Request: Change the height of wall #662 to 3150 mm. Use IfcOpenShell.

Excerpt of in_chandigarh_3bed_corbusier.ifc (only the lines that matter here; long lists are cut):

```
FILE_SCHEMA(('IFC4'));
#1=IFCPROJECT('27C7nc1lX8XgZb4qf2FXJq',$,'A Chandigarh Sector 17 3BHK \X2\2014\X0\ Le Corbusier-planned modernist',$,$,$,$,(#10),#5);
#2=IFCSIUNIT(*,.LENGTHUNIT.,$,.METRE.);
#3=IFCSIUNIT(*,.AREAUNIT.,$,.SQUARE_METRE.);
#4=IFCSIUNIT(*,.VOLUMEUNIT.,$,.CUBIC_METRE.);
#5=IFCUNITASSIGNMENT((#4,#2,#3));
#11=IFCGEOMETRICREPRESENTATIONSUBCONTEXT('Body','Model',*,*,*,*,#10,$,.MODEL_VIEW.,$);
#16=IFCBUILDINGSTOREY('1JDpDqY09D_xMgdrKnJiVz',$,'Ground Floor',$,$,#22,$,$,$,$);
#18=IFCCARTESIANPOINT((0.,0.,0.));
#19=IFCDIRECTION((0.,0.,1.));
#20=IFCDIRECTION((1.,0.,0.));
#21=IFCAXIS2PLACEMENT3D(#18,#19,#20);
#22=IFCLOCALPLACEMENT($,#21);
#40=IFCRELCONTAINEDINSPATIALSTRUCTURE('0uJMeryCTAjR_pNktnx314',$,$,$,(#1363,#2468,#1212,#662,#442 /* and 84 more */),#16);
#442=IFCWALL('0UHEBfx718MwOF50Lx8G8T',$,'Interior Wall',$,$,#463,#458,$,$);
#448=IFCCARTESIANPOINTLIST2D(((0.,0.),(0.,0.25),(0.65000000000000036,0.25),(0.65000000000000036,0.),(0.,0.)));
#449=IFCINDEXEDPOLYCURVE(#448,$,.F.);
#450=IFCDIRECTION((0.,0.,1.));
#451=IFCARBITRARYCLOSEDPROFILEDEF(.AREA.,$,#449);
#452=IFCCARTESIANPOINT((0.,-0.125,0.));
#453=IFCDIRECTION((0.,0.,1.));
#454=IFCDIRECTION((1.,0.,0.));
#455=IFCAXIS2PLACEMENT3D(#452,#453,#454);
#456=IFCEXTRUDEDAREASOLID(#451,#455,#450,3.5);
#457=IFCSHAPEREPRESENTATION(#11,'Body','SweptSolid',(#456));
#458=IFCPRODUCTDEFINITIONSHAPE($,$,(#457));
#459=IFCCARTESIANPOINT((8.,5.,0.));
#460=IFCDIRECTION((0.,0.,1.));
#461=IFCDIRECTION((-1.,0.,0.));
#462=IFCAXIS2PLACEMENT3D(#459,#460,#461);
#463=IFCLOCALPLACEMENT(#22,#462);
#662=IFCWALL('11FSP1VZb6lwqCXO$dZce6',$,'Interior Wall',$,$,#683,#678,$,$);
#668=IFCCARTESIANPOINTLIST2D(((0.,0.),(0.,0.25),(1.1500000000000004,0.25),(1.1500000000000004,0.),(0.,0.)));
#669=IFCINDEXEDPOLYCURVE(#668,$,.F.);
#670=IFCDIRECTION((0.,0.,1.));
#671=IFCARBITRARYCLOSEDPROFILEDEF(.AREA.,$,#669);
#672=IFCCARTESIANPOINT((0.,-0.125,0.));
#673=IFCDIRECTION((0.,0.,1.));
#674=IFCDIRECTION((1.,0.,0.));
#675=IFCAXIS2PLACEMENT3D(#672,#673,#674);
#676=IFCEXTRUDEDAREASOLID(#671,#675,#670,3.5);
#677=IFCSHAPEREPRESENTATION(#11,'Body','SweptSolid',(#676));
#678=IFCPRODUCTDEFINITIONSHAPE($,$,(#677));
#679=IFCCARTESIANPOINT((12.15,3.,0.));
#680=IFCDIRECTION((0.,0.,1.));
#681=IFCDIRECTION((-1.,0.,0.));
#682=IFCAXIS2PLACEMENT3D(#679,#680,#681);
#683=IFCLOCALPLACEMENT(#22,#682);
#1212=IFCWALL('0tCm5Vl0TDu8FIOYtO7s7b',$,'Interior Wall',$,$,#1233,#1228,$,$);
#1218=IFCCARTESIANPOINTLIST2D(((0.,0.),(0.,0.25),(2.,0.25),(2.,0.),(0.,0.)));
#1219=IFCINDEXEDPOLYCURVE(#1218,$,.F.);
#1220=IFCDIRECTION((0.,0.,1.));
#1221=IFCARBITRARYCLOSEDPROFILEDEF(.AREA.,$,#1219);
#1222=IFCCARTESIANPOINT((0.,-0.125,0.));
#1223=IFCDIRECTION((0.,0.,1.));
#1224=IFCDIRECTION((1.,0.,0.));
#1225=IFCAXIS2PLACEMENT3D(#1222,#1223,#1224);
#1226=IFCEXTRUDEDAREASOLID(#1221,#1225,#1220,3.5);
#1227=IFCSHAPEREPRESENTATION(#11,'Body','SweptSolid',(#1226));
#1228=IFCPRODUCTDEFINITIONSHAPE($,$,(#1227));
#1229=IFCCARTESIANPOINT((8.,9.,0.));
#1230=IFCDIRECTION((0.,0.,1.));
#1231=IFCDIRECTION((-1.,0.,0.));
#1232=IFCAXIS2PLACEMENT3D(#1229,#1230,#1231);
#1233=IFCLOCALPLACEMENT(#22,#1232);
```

```python
import ifcopenshell
import ifcopenshell.geom
import ifcopenshell.util.representation
import ifcopenshell.util.shape

model = ifcopenshell.open("in_chandigarh_3bed_corbusier.ifc")
settings = ifcopenshell.geom.settings()


def volume(element):
    """Net volume in cubic metres, openings subtracted."""
    shape = ifcopenshell.geom.create_shape(settings, element)
    return ifcopenshell.util.shape.get_volume(shape.geometry)


wall = model.by_guid("11FSP1VZb6lwqCXO$dZce6")
before = volume(wall)

body = ifcopenshell.util.representation.get_representation(wall, "Model", "Body")
solid = body.Items[0]
old_height = solid.Depth
solid.Depth = 3.15
after = volume(wall)

print(f"height {old_height:g} -> {solid.Depth:g}, volume {before:.3f} -> {after:.3f} m3")

model.write("in_chandigarh_3bed_corbusier-out.ifc")
```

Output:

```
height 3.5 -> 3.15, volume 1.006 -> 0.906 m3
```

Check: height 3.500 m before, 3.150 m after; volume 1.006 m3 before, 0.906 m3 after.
